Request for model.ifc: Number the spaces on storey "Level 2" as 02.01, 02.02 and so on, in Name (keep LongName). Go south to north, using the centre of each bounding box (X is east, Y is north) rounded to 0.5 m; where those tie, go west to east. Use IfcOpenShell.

First a look at what the model holds.

```python
import ifcopenshell
import ifcopenshell.util.element
import ifcopenshell.util.placement

model = ifcopenshell.open("model.ifc")
print(model.schema)
storey = next(s for s in model.by_type("IfcBuildingStorey") if s.Name == "Level 2")
spaces = [e for e in ifcopenshell.util.element.get_decomposition(storey) if e.is_a("IfcSpace")]
for e in sorted(spaces, key=lambda e: e.id()):
    origin = ifcopenshell.util.placement.get_local_placement(e.ObjectPlacement)[:3, 3]
    print(e.id(), e.Name, e.LongName, origin.round(2) + 0.0, sep=" | ")
```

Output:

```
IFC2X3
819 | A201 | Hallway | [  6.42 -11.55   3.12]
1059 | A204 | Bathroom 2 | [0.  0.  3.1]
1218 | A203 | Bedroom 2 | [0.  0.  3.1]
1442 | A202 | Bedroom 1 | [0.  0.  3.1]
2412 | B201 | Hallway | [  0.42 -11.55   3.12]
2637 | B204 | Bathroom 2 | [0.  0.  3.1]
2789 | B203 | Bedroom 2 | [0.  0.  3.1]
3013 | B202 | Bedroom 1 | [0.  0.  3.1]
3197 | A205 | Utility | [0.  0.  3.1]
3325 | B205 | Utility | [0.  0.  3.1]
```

```python
import ifcopenshell
import ifcopenshell.geom
import ifcopenshell.util.element
import ifcopenshell.util.shape

model = ifcopenshell.open("model.ifc")
settings = ifcopenshell.geom.settings()
settings.set("use-world-coords", True)


def centre(element):
    shape = ifcopenshell.geom.create_shape(settings, element)
    return ifcopenshell.util.shape.get_bbox_centroid(shape.geometry)


storey = next(s for s in model.by_type("IfcBuildingStorey") if s.Name == "Level 2")
spaces = [e for e in ifcopenshell.util.element.get_decomposition(storey) if e.is_a("IfcSpace")]

# Insertion points can sit at a corner or the storey origin, so sort by the geometry (in metres).
centres = {e: centre(e) for e in spaces}
spaces.sort(key=lambda e: (round(centres[e][1] / 0.5), centres[e][0]))

for i, e in enumerate(spaces, start=1):
    number = f"02.{i:02d}"
    e.Name = number
    print(e.id(), number)

model.write("model-out.ifc")
```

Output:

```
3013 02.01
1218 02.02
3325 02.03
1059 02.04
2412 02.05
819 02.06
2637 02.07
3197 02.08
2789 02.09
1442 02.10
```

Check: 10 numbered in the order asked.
